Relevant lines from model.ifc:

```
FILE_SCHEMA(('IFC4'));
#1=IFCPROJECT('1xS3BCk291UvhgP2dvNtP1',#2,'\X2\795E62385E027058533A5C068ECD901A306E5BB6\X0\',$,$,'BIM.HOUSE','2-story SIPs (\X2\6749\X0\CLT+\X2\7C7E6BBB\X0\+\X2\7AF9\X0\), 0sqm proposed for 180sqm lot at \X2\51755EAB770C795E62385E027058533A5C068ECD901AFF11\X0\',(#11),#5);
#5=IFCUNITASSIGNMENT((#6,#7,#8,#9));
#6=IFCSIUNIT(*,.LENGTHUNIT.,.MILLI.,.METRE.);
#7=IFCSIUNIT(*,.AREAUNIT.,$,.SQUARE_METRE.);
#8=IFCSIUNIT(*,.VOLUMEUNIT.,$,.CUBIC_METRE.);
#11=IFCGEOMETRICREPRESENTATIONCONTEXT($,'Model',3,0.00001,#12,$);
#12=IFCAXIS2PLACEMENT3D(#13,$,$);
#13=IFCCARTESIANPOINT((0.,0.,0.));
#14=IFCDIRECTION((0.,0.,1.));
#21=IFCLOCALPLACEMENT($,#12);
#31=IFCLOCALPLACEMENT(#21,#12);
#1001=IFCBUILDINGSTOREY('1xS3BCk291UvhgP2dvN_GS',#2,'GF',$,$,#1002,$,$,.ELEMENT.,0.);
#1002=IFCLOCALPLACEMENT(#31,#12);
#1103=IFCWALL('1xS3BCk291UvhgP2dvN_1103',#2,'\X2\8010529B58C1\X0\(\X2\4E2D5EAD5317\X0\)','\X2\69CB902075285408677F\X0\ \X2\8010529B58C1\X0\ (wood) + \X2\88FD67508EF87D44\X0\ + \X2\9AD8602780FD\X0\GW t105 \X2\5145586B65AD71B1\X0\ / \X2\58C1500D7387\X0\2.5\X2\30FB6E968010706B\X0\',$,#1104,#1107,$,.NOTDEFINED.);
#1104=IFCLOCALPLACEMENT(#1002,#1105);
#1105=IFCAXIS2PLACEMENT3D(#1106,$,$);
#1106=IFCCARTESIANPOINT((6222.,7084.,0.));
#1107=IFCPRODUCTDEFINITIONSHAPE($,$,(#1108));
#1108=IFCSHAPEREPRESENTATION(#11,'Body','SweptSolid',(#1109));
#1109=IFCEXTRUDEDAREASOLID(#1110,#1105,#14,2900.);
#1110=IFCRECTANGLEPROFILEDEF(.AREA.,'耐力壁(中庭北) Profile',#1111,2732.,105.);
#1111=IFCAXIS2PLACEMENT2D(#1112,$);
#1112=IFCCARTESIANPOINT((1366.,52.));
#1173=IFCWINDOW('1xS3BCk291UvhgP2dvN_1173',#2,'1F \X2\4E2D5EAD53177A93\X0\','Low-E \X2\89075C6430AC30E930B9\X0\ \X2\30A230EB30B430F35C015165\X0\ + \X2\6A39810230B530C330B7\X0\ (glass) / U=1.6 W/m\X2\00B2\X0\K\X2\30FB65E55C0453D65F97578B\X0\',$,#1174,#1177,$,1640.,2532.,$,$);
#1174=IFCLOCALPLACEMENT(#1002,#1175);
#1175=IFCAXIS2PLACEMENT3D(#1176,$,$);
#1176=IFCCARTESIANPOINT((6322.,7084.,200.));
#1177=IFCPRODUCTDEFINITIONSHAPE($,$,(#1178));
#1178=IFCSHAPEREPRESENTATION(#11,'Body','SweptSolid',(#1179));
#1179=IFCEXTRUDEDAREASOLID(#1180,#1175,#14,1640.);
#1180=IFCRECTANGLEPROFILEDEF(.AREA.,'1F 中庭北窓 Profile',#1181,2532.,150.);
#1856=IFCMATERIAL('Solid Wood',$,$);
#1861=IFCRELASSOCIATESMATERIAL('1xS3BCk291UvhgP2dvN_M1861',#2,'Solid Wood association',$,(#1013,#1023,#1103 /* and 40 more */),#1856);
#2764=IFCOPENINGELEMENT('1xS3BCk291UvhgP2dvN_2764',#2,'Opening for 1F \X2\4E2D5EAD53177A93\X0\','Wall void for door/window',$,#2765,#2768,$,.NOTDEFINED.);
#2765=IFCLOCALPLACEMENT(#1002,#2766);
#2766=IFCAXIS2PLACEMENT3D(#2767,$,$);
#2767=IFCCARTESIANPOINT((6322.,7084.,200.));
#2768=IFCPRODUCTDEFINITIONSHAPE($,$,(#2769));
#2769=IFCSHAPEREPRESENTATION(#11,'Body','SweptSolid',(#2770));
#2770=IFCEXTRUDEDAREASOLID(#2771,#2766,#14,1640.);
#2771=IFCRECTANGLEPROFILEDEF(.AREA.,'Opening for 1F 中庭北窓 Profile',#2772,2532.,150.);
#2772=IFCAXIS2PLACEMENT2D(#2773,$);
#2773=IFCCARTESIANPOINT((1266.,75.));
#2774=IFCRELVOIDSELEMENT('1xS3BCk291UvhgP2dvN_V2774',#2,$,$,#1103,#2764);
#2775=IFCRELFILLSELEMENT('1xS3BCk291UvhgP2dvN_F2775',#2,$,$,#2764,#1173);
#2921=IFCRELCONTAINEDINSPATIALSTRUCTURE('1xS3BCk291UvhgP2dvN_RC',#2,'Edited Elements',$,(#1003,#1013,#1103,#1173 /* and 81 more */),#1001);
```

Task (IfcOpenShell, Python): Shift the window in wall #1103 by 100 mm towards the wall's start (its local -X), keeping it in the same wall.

```python
import ifcopenshell
import ifcopenshell.api.geometry
import ifcopenshell.util.placement
import ifcopenshell.util.unit

model = ifcopenshell.open("model.ifc")
unit_scale = ifcopenshell.util.unit.calculate_unit_scale(model)

window = model.by_guid("1xS3BCk291UvhgP2dvN_1173")
opening = window.FillsVoids[0].RelatingOpeningElement
wall = opening.VoidsElements[0].RelatingBuildingElement

wall_matrix = ifcopenshell.util.placement.get_local_placement(wall.ObjectPlacement)
shift = wall_matrix[:3, 0] * -0.1 / unit_scale
before = ifcopenshell.util.placement.get_local_placement(window.ObjectPlacement)[:3, 3].copy()

# The window is not placed relative to its opening, so move both.
for product in (opening, window):
    matrix = ifcopenshell.util.placement.get_local_placement(product.ObjectPlacement)
    matrix[:3, 3] += shift
    ifcopenshell.api.geometry.edit_object_placement(model, product=product, matrix=matrix, is_si=False)

after = ifcopenshell.util.placement.get_local_placement(window.ObjectPlacement)[:3, 3]
print("window moved by", (after - before).round(3) + 0.0)

model.write("model_edited.ifc")
```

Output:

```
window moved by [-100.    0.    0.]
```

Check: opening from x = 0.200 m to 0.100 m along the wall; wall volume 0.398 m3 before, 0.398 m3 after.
